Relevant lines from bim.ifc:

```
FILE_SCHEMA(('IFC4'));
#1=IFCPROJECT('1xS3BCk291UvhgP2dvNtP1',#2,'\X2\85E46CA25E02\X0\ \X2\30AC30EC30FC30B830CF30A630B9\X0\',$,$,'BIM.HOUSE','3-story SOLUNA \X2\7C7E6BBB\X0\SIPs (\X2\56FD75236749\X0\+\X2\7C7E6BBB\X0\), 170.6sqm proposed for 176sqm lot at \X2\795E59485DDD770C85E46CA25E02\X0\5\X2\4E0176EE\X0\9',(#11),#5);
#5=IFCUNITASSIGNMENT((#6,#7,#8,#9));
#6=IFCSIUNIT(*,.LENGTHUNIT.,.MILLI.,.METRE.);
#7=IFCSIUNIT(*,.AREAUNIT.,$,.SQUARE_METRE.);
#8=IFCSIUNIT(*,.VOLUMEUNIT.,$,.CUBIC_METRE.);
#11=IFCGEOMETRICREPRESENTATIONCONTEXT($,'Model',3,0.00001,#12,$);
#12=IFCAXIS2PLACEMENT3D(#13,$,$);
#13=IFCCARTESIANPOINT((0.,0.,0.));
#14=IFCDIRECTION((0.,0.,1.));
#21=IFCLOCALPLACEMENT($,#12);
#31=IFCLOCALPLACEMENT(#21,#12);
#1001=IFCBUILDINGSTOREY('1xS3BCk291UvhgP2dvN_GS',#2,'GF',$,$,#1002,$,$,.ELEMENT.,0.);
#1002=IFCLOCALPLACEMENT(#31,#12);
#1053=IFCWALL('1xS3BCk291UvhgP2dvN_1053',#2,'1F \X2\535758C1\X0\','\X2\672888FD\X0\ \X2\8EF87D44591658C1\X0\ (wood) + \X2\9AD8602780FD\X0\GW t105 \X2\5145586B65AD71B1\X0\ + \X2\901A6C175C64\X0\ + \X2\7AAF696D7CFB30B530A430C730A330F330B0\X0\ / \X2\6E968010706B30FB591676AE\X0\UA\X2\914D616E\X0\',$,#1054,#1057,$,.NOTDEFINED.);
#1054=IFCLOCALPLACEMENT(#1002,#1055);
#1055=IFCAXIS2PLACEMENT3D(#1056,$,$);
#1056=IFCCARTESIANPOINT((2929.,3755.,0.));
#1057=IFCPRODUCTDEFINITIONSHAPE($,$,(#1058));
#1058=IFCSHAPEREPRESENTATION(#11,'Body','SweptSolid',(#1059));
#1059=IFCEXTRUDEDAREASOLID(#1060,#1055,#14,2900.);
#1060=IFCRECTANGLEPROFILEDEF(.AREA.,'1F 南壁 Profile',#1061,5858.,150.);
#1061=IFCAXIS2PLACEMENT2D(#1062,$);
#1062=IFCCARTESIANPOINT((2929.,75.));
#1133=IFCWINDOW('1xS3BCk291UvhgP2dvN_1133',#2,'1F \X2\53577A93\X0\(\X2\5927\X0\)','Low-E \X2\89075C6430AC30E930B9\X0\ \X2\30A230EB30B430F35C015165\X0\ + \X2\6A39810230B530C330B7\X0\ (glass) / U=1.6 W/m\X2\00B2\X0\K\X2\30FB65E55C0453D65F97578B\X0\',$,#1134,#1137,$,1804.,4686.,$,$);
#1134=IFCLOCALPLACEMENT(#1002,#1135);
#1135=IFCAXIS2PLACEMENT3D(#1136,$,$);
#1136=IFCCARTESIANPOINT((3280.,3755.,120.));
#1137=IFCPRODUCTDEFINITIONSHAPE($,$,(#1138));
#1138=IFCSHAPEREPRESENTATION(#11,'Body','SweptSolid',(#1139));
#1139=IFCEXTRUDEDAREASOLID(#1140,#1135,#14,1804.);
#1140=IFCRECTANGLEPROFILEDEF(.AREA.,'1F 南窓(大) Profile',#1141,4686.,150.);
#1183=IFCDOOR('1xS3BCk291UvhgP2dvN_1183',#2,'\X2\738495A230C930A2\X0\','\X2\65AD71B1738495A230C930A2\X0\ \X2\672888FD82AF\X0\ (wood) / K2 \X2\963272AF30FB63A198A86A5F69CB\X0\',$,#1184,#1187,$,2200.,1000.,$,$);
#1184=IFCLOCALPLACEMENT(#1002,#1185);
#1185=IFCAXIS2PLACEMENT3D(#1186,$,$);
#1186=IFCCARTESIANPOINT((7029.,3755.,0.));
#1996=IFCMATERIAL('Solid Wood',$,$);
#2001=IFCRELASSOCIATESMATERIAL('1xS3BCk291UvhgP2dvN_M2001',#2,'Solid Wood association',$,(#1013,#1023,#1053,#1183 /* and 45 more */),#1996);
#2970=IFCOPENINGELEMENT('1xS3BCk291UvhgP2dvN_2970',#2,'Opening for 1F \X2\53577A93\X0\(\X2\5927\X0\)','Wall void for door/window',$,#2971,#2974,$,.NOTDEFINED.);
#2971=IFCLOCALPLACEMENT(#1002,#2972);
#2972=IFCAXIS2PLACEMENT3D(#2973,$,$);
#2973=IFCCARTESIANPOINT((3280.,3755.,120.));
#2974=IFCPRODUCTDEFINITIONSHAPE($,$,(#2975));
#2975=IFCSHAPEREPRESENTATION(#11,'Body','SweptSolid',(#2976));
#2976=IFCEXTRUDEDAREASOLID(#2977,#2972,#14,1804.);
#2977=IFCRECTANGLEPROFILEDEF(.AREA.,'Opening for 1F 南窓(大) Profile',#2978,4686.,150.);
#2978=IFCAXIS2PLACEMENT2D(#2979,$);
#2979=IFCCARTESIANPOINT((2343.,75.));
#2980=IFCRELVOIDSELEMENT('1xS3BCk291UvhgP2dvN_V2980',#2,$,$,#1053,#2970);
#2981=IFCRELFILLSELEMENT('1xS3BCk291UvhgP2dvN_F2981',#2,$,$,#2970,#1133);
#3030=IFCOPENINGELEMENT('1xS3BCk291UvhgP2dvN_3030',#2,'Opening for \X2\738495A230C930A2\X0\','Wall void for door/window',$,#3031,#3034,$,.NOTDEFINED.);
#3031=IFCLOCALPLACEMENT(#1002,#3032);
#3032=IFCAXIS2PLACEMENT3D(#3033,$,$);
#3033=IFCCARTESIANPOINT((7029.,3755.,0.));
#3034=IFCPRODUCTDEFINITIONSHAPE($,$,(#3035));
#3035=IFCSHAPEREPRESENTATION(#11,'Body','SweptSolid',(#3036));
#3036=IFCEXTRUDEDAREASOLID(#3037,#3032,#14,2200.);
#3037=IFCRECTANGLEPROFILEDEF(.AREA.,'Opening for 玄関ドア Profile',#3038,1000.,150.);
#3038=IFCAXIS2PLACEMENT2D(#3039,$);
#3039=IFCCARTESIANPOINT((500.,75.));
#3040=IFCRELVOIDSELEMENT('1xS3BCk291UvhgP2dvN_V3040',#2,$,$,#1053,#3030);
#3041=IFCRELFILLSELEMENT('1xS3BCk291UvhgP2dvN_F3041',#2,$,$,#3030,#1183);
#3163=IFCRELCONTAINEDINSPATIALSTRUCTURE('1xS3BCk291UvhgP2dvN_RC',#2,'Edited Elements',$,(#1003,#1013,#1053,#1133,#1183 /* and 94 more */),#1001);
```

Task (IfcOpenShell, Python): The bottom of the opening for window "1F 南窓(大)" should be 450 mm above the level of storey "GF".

```python
import numpy as np
import ifcopenshell
import ifcopenshell.api.geometry
import ifcopenshell.geom
import ifcopenshell.util.element
import ifcopenshell.util.placement
import ifcopenshell.util.shape
import ifcopenshell.util.unit

model = ifcopenshell.open("bim.ifc")
unit_scale = ifcopenshell.util.unit.calculate_unit_scale(model)

window = model.by_guid("1xS3BCk291UvhgP2dvN_1133")
opening = window.FillsVoids[0].RelatingOpeningElement
storey = ifcopenshell.util.element.get_container(window, ifc_class="IfcBuildingStorey")
level = ifcopenshell.util.placement.get_local_placement(storey.ObjectPlacement)[2, 3]

# The opening's origin need not be at the sill, so measure its lowest point.
shape = ifcopenshell.geom.create_shape(ifcopenshell.geom.settings(), opening)
bottom = ifcopenshell.util.shape.get_shape_bottom_elevation(shape, shape.geometry) / unit_scale
dz = level + 0.45 / unit_scale - bottom

shift = np.array([0.0, 0.0, dz])
# The window is not placed relative to its opening, so move both.
for product in (opening, window):
    matrix = ifcopenshell.util.placement.get_local_placement(product.ObjectPlacement)
    matrix[:3, 3] += shift
    ifcopenshell.api.geometry.edit_object_placement(model, product=product, matrix=matrix, is_si=False)

print(f"moved by {dz * unit_scale:+.3f} m")

model.write("bim-out.ifc")
```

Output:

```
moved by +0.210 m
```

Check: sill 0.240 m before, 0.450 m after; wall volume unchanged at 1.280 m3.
